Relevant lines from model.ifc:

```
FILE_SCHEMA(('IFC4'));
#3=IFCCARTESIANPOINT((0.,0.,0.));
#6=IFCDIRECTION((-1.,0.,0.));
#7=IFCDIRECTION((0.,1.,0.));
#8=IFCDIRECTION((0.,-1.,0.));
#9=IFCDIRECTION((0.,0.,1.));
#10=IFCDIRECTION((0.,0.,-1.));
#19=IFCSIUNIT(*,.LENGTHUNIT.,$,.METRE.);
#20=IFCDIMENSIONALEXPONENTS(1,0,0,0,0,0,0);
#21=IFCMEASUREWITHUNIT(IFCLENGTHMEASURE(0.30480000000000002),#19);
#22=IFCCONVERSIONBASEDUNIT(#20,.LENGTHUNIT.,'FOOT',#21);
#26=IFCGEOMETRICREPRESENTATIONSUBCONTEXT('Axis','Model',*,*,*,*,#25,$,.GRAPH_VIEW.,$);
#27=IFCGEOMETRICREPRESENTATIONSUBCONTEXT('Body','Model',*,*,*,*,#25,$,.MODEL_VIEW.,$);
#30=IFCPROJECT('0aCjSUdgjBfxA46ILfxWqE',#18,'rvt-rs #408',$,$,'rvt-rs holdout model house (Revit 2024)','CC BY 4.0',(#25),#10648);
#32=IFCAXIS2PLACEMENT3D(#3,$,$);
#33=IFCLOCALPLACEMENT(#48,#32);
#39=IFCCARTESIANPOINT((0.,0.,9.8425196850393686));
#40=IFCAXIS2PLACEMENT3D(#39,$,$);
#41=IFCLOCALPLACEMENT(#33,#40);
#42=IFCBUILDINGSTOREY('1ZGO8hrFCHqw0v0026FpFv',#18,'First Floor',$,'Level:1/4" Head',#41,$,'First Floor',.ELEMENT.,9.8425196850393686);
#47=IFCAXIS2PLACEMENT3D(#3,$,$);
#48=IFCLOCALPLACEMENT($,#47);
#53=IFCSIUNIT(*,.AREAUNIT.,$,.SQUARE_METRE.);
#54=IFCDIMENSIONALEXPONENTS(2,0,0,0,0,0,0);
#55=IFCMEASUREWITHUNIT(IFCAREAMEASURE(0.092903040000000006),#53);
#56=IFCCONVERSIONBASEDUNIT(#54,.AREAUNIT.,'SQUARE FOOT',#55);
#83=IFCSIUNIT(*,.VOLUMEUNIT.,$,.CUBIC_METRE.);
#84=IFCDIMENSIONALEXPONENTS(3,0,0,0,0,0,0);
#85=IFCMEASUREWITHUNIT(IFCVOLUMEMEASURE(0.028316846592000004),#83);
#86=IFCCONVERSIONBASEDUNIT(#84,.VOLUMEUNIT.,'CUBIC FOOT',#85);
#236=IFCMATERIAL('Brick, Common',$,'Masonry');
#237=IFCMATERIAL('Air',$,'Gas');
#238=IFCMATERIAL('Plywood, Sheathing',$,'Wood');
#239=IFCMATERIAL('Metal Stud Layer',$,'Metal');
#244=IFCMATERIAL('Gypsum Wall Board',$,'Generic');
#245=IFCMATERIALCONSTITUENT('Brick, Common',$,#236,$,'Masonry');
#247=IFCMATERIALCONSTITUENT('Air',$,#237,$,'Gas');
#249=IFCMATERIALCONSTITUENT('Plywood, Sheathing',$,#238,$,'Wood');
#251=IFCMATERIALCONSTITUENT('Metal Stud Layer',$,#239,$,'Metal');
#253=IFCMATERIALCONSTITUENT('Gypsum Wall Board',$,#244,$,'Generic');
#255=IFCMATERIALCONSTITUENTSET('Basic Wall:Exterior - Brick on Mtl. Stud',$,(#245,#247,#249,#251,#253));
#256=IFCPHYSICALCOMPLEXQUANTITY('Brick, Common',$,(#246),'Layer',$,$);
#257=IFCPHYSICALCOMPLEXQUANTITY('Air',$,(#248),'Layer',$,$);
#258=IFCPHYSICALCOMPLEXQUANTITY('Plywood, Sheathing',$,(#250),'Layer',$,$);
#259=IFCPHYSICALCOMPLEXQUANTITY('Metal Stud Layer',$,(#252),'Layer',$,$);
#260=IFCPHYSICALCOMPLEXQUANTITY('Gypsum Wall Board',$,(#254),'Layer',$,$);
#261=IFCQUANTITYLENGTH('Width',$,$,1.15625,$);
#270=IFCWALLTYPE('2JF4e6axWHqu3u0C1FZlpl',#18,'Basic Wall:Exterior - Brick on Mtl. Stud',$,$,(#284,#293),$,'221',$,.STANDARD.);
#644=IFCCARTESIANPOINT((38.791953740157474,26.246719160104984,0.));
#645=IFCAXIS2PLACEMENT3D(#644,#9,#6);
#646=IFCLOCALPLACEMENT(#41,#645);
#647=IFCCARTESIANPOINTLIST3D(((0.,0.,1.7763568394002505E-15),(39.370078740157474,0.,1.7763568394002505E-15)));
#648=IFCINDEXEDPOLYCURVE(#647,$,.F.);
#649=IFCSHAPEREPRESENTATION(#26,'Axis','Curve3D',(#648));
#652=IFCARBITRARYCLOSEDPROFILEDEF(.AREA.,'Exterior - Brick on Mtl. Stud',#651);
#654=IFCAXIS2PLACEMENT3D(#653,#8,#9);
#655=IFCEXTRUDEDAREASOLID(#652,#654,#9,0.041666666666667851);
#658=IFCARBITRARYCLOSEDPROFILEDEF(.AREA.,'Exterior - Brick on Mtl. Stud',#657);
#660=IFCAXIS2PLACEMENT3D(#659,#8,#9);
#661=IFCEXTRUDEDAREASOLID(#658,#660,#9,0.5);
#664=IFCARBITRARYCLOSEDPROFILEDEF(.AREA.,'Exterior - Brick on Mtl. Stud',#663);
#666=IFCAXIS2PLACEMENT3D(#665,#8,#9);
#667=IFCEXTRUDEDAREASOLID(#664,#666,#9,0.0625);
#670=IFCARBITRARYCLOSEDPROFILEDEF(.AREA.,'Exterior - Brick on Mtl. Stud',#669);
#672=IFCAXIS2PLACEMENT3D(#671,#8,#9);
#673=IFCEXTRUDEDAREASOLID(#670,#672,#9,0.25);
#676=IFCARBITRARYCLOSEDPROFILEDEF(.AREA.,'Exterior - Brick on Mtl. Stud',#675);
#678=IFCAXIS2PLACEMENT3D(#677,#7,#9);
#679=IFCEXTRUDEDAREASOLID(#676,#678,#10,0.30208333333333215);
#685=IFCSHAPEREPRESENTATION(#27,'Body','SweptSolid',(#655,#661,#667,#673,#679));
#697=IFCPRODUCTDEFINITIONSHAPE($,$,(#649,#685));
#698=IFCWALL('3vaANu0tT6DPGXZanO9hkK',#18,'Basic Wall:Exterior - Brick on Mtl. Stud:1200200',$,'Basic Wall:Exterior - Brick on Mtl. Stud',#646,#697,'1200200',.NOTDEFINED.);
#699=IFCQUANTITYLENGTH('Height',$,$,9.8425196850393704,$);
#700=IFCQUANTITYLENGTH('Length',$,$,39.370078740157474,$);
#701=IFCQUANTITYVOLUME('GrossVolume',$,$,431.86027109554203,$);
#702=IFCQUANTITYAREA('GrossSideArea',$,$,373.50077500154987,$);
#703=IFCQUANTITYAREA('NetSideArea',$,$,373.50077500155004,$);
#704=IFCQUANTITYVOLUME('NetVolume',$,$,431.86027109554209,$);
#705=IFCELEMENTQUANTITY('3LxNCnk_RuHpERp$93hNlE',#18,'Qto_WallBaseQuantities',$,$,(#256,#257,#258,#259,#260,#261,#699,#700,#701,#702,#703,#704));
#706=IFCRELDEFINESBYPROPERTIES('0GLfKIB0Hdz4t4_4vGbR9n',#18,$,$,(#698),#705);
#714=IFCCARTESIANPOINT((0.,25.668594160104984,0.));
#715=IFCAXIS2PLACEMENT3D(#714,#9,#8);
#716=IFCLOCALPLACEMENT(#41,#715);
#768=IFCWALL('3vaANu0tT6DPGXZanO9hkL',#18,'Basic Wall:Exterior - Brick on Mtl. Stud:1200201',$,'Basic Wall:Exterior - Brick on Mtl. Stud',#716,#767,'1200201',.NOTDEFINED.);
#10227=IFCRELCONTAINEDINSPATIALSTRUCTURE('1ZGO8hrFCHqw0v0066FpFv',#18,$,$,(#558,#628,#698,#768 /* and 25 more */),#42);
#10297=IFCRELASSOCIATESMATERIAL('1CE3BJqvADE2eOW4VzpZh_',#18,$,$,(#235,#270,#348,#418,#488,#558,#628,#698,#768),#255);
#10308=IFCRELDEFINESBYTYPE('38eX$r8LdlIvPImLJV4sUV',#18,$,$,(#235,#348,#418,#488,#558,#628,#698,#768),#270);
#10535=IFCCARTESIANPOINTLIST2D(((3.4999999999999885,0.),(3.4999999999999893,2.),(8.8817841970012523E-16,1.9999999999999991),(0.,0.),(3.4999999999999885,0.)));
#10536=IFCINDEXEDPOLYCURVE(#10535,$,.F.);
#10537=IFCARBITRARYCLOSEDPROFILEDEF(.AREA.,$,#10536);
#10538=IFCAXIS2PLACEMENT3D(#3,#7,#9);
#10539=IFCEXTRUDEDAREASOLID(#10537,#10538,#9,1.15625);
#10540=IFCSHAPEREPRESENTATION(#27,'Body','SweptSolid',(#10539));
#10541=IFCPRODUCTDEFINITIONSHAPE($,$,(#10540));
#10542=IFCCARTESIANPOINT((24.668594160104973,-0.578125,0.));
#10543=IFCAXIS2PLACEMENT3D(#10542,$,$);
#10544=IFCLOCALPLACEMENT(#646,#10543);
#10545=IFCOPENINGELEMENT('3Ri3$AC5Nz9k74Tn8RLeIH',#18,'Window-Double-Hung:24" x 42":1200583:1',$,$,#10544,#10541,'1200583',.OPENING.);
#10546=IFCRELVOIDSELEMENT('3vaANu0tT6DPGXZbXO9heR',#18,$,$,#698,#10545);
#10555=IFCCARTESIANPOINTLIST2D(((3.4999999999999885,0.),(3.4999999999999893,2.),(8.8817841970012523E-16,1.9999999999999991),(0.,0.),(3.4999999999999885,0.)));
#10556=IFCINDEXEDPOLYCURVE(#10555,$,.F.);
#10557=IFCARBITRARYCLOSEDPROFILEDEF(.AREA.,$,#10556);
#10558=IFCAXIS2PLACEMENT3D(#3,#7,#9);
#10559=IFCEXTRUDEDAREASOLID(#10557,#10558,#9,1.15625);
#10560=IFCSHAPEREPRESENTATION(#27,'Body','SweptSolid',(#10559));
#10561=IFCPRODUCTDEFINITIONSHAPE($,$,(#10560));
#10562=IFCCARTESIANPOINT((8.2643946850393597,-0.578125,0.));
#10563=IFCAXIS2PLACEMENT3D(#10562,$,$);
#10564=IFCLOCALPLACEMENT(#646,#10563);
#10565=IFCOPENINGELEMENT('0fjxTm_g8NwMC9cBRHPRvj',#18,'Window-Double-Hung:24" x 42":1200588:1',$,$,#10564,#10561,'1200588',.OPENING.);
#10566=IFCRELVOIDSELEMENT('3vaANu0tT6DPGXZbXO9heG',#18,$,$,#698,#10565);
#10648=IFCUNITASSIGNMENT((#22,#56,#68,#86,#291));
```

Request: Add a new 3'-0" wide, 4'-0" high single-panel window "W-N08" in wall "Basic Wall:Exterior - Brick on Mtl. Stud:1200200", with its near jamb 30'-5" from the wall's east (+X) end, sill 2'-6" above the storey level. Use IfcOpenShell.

```python
import numpy as np
import ifcopenshell
import ifcopenshell.api.feature
import ifcopenshell.api.geometry
import ifcopenshell.api.pset
import ifcopenshell.api.root
import ifcopenshell.api.spatial
import ifcopenshell.geom
import ifcopenshell.util.element
import ifcopenshell.util.placement
import ifcopenshell.util.representation
import ifcopenshell.util.shape
import ifcopenshell.util.unit

model = ifcopenshell.open("model.ifc")
unit_scale = ifcopenshell.util.unit.calculate_unit_scale(model)
area_scale = ifcopenshell.util.unit.calculate_unit_scale(model, "AREAUNIT")
volume_scale = ifcopenshell.util.unit.calculate_unit_scale(model, "VOLUMEUNIT")
settings = ifcopenshell.geom.settings()


def volume(element):
    """Net volume in cubic metres, openings subtracted."""
    shape = ifcopenshell.geom.create_shape(settings, element)
    return ifcopenshell.util.shape.get_volume(shape.geometry)


wall = model.by_guid("3vaANu0tT6DPGXZanO9hkK")
storey = ifcopenshell.util.element.get_container(wall, ifc_class="IfcBuildingStorey")
context = ifcopenshell.util.representation.get_context(model, "Model", "Body", "MODEL_VIEW")
before = volume(wall)

width, height, from_end, sill = 0.9144, 1.2192, 9.271, 0.762  # metres

# The wall runs along its own X axis, and the end named is its -X end.
wall_shape = ifcopenshell.geom.create_shape(settings, wall)
x, y, z = ifcopenshell.util.shape.get_vertices(wall_shape.geometry).T
start = x.min() + from_end
face, thickness = float(y.min()), float(y.max() - y.min())
wall_matrix = ifcopenshell.util.placement.get_local_placement(wall.ObjectPlacement)
level = ifcopenshell.util.placement.get_local_placement(storey.ObjectPlacement)[2, 3]


def in_wall(x, y):
    """Placement at x, y metres in the wall's axes, at sill height."""
    matrix = wall_matrix.copy()
    matrix[:, 3] = wall_matrix @ np.array([x / unit_scale, y / unit_scale, 0.0, 1.0])
    matrix[2, 3] = level + sill / unit_scale
    return matrix


# Opening: a box that overshoots both wall faces by 50 mm.
opening = ifcopenshell.api.root.create_entity(model, ifc_class="IfcOpeningElement", predefined_type="OPENING")
box = ifcopenshell.api.geometry.add_wall_representation(
    model, context=context, length=width, height=height, thickness=thickness + 0.1
)
ifcopenshell.api.geometry.assign_representation(model, product=opening, representation=box)
ifcopenshell.api.geometry.edit_object_placement(model, product=opening, matrix=in_wall(start, face - 0.05), is_si=False)
ifcopenshell.api.feature.add_feature(model, feature=opening, element=wall)

window = ifcopenshell.api.root.create_entity(model, ifc_class="IfcWindow", name="W-N08", predefined_type="WINDOW")
window.OverallWidth, window.OverallHeight = width / unit_scale, height / unit_scale
window.PartitioningType = "SINGLE_PANEL"
body = ifcopenshell.api.geometry.add_window_representation(
    model,
    context=context,
    overall_width=window.OverallWidth,
    overall_height=window.OverallHeight,
    partition_type="SINGLE_PANEL",
)
ifcopenshell.api.geometry.assign_representation(model, product=window, representation=body)
ifcopenshell.api.spatial.assign_container(model, products=[window], relating_structure=storey)
ifcopenshell.api.feature.add_filling(model, opening=opening, element=window)

# Centre the window in the wall's thickness.
ifcopenshell.api.geometry.edit_object_placement(model, product=window, matrix=in_wall(start, face), is_si=False)
window_shape = ifcopenshell.geom.create_shape(settings, window)
depth = ifcopenshell.util.shape.get_vertices(window_shape.geometry)[:, 1]
offset = face + thickness / 2 - (depth.min() + depth.max()) / 2
ifcopenshell.api.geometry.edit_object_placement(model, product=window, matrix=in_wall(start, offset), is_si=False)

after = volume(wall)

# Update the wall's stored quantities.
qto = model.by_id(ifcopenshell.util.element.get_pset(wall, "Qto_WallBaseQuantities", should_inherit=False)["id"])
ifcopenshell.api.pset.edit_qto(model, qto=qto, properties={
    "NetSideArea": after / thickness / area_scale,
    "NetVolume": after / volume_scale,
})

print(f"wall volume {before:.3f} -> {after:.3f} m3")

model.write("model-out.ifc")
```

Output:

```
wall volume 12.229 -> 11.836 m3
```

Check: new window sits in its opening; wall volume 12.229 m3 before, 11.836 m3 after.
